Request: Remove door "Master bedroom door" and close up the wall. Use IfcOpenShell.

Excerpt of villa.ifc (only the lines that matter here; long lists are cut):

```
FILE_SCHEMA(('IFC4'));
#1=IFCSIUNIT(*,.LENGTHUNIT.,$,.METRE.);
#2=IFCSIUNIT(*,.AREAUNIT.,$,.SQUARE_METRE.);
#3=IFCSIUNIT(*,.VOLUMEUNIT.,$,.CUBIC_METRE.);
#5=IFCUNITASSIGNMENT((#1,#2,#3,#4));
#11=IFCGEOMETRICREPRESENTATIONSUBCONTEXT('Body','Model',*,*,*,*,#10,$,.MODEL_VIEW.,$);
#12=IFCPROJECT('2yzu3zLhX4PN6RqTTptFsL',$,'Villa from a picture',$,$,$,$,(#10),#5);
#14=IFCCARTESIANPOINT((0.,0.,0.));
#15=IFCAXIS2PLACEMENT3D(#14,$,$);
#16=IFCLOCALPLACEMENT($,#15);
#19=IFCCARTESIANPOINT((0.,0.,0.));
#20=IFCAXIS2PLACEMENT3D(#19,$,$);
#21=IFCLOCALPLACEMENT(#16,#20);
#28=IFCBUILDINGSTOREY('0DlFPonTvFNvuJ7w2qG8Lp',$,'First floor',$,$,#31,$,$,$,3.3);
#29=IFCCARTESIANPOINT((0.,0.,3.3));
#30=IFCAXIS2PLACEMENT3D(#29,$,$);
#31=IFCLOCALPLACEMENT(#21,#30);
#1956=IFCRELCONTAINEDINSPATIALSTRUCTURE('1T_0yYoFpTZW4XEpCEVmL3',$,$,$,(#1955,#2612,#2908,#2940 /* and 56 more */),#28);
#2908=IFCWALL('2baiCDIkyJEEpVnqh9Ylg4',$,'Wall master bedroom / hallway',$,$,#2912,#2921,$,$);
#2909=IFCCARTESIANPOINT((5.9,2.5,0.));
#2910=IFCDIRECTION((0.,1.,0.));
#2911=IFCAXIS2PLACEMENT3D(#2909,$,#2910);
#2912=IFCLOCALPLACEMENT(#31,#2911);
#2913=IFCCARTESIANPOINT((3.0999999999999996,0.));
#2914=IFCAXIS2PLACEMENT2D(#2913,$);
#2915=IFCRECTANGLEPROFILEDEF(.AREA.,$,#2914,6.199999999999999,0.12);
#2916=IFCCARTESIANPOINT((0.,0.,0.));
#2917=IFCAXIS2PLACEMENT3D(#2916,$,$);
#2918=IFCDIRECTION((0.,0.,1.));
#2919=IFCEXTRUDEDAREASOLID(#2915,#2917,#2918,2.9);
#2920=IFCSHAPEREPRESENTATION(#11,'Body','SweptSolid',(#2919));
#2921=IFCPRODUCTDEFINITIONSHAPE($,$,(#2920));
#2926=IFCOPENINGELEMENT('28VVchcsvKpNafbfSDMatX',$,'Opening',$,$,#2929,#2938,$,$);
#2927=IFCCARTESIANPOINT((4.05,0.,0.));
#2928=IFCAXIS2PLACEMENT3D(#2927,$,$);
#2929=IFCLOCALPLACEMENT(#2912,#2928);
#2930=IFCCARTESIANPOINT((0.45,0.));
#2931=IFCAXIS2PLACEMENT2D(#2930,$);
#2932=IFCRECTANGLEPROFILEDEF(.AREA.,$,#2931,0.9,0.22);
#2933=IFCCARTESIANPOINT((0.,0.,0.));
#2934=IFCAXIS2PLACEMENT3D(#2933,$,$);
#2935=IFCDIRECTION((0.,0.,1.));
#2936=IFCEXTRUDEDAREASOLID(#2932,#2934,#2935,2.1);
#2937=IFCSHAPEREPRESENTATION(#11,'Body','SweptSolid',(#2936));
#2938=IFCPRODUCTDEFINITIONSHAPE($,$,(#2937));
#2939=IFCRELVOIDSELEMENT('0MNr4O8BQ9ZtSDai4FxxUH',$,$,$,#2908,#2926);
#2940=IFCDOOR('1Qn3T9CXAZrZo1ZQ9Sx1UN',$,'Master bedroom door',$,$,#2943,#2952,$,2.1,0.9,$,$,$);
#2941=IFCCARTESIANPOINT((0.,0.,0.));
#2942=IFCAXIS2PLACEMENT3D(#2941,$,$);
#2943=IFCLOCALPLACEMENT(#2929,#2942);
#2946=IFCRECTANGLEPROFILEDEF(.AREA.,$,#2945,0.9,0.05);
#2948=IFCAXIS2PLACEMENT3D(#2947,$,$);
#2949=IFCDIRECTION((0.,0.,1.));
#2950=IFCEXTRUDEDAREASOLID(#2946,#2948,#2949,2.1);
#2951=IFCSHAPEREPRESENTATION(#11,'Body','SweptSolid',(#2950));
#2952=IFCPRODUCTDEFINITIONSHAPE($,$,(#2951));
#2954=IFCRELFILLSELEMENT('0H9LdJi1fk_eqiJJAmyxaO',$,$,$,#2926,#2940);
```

```python
import ifcopenshell
import ifcopenshell.api.feature
import ifcopenshell.api.root
import ifcopenshell.geom
import ifcopenshell.util.shape

model = ifcopenshell.open("villa.ifc")
settings = ifcopenshell.geom.settings()


def volume(element):
    """Net volume in cubic metres, openings subtracted."""
    shape = ifcopenshell.geom.create_shape(settings, element)
    return ifcopenshell.util.shape.get_volume(shape.geometry)


door = model.by_guid("1Qn3T9CXAZrZo1ZQ9Sx1UN")
opening = door.FillsVoids[0].RelatingOpeningElement
wall = opening.VoidsElements[0].RelatingBuildingElement
before = volume(wall)

ifcopenshell.api.root.remove_product(model, product=door)
ifcopenshell.api.feature.remove_feature(model, feature=opening)

after = volume(wall)

print(f"wall volume {before:.3f} -> {after:.3f} m3")

model.write("villa_v2.ifc")
```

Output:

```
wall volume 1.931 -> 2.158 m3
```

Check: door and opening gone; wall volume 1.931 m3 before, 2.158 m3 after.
